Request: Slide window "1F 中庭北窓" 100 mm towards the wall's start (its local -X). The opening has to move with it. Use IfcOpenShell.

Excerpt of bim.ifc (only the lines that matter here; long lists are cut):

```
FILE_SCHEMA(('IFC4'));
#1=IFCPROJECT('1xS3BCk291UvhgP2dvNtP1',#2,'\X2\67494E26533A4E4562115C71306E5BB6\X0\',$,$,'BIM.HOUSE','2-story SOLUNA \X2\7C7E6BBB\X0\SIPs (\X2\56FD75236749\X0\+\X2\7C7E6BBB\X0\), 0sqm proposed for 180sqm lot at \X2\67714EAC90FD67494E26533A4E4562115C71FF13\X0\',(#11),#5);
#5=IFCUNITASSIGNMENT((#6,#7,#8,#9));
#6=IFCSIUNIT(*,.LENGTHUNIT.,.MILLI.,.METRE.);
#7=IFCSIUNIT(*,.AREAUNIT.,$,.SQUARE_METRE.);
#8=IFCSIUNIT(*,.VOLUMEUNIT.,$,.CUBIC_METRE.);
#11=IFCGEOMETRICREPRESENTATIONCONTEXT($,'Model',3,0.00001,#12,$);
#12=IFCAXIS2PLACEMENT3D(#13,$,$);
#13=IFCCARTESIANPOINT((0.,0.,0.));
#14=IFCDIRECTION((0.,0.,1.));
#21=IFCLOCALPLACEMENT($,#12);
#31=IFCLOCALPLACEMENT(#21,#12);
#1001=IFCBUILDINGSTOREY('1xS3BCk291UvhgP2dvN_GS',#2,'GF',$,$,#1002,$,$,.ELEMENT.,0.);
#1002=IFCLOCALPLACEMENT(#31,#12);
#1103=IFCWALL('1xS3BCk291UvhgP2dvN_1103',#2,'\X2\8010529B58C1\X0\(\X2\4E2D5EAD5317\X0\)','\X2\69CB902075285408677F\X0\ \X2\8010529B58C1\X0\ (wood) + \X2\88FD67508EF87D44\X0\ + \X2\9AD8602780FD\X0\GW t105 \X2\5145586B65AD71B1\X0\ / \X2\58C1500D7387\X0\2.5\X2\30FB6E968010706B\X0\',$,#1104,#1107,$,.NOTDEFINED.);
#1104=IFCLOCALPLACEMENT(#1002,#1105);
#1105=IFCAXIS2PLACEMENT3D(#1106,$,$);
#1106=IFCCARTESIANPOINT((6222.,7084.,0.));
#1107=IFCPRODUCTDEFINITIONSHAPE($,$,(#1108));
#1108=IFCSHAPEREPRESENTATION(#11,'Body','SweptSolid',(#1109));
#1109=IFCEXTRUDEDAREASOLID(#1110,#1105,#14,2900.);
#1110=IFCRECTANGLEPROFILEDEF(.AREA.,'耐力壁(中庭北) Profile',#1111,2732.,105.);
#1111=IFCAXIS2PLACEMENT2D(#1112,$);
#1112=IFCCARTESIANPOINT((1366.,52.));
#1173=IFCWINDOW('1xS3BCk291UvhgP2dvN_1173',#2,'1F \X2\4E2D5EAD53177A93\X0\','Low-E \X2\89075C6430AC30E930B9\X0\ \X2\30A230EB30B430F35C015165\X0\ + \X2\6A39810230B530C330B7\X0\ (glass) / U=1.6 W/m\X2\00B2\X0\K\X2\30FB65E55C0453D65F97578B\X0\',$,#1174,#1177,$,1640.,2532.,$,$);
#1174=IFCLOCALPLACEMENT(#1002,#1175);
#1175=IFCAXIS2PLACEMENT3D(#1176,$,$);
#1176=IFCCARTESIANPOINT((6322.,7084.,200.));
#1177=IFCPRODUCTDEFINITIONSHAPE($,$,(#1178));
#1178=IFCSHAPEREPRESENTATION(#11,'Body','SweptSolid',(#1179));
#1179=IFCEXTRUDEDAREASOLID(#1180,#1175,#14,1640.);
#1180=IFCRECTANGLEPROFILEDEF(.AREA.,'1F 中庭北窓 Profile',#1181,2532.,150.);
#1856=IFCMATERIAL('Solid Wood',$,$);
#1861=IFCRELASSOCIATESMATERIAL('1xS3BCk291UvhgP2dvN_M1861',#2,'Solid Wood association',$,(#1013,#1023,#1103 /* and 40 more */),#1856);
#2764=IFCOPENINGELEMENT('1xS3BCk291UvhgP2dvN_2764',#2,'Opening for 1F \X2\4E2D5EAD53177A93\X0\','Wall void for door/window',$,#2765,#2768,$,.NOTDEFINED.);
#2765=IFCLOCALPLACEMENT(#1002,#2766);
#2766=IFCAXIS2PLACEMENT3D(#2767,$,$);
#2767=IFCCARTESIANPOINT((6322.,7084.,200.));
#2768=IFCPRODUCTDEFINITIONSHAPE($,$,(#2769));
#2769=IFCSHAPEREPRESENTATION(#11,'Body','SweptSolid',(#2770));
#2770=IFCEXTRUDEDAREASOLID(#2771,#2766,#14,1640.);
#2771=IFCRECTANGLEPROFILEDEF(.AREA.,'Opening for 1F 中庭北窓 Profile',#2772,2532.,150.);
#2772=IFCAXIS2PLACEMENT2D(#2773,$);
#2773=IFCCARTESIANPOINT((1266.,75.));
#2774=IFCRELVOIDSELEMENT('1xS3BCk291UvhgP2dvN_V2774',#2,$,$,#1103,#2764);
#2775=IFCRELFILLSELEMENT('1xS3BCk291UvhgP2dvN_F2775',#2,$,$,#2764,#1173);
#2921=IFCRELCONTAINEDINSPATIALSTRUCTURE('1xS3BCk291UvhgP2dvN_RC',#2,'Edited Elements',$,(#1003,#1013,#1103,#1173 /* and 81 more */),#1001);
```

```python
import ifcopenshell
import ifcopenshell.api.geometry
import ifcopenshell.util.placement

model = ifcopenshell.open("bim.ifc")

window = model.by_guid("1xS3BCk291UvhgP2dvN_1173")
opening = window.FillsVoids[0].RelatingOpeningElement
wall = opening.VoidsElements[0].RelatingBuildingElement

wall_matrix = ifcopenshell.util.placement.get_local_placement(wall.ObjectPlacement)
shift = wall_matrix[:3, 0] * -100.0
before = ifcopenshell.util.placement.get_local_placement(window.ObjectPlacement)[:3, 3].copy()

# The window is not placed relative to its opening, so move both.
for product in (opening, window):
    matrix = ifcopenshell.util.placement.get_local_placement(product.ObjectPlacement)
    matrix[:3, 3] += shift
    ifcopenshell.api.geometry.edit_object_placement(model, product=product, matrix=matrix, is_si=False)

after = ifcopenshell.util.placement.get_local_placement(window.ObjectPlacement)[:3, 3]
print("window moved by", (after - before).round(3) + 0.0)

model.write("bim_updated.ifc")
```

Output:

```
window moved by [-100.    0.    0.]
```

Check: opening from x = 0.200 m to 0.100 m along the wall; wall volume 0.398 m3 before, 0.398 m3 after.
